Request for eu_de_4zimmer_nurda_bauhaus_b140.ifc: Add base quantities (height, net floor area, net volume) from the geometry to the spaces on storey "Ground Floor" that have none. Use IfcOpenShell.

First a look at what the model holds.

```python
import ifcopenshell
import ifcopenshell.util.element
import ifcopenshell.util.unit

model = ifcopenshell.open("eu_de_4zimmer_nurda_bauhaus_b140.ifc")
print(model.schema)
for unit_type in ("LENGTHUNIT", "AREAUNIT", "VOLUMEUNIT"):
    print(unit_type, ifcopenshell.util.unit.calculate_unit_scale(model, unit_type))
storey = next(s for s in model.by_type("IfcBuildingStorey") if s.Name == "Ground Floor")
spaces = [e for e in ifcopenshell.util.element.get_decomposition(storey) if e.is_a("IfcSpace")]
for e in sorted(spaces, key=lambda e: e.id()):
    print(e.id(), e.is_a(), e.Name, list(ifcopenshell.util.element.get_psets(e, qtos_only=True)), sep=" | ")
```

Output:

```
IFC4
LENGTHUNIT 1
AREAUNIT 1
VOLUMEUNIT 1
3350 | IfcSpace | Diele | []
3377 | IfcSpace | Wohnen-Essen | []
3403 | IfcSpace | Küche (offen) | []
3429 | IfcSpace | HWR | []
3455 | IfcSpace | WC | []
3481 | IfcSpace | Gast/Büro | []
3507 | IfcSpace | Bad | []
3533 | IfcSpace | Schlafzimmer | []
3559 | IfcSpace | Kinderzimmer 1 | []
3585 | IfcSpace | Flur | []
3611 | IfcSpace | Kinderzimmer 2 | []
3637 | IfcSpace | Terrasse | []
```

```python
import ifcopenshell
import ifcopenshell.api.pset
import ifcopenshell.geom
import ifcopenshell.util.element
import ifcopenshell.util.shape
import ifcopenshell.util.unit

model = ifcopenshell.open("eu_de_4zimmer_nurda_bauhaus_b140.ifc")
unit_scale = ifcopenshell.util.unit.calculate_unit_scale(model)
area_scale = ifcopenshell.util.unit.calculate_unit_scale(model, "AREAUNIT")
volume_scale = ifcopenshell.util.unit.calculate_unit_scale(model, "VOLUMEUNIT")
settings = ifcopenshell.geom.settings()

storey = next(s for s in model.by_type("IfcBuildingStorey") if s.Name == "Ground Floor")
spaces = [e for e in ifcopenshell.util.element.get_decomposition(storey) if e.is_a("IfcSpace")]

for e in sorted(spaces, key=lambda e: e.id()):
    if ifcopenshell.util.element.get_psets(e, qtos_only=True, should_inherit=False):
        continue
    # Geometry comes back in metres, in the element's own axes.
    shape = ifcopenshell.geom.create_shape(settings, e)
    values = {
        "Height": ifcopenshell.util.shape.get_z(shape.geometry) / unit_scale,
        "NetFloorArea": ifcopenshell.util.shape.get_footprint_area(shape.geometry) / area_scale,
        "NetVolume": ifcopenshell.util.shape.get_volume(shape.geometry) / volume_scale,
    }
    qto = ifcopenshell.api.pset.add_qto(model, product=e, name="Qto_SpaceBaseQuantities")
    ifcopenshell.api.pset.edit_qto(model, qto=qto, properties=values)
    print(e.id(), {k: round(v, 3) for k, v in values.items()})

model.write("eu_de_4zimmer_nurda_bauhaus_b140_v2.ifc")
```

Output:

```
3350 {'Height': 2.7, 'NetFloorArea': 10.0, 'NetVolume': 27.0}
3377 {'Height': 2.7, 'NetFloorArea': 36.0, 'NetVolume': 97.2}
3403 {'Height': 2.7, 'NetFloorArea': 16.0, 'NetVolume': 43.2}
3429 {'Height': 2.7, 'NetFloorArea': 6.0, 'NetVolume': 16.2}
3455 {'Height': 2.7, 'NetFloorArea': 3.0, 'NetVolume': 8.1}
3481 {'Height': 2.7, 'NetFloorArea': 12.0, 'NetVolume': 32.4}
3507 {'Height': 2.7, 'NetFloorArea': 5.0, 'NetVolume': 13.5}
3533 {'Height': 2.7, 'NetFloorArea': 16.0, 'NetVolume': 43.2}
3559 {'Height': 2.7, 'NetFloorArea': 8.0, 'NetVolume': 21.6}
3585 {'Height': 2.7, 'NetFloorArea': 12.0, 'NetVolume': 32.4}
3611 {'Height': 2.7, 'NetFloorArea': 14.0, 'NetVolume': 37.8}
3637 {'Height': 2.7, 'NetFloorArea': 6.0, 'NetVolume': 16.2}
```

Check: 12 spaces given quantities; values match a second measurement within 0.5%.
